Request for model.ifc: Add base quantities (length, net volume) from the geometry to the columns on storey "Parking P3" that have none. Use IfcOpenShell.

First a look at what the model holds.

```python
import ifcopenshell
import ifcopenshell.util.element
import ifcopenshell.util.unit

model = ifcopenshell.open("model.ifc")
print(model.schema)
for unit_type in ("LENGTHUNIT", "AREAUNIT", "VOLUMEUNIT"):
    print(unit_type, ifcopenshell.util.unit.calculate_unit_scale(model, unit_type))
storey = next(s for s in model.by_type("IfcBuildingStorey") if s.Name == "Parking P3")
columns = [e for e in ifcopenshell.util.element.get_decomposition(storey) if e.is_a("IfcColumn")]
for e in sorted(columns, key=lambda e: e.id()):
    print(e.id(), e.is_a(), e.Name, list(ifcopenshell.util.element.get_psets(e, qtos_only=True)), sep=" | ")
```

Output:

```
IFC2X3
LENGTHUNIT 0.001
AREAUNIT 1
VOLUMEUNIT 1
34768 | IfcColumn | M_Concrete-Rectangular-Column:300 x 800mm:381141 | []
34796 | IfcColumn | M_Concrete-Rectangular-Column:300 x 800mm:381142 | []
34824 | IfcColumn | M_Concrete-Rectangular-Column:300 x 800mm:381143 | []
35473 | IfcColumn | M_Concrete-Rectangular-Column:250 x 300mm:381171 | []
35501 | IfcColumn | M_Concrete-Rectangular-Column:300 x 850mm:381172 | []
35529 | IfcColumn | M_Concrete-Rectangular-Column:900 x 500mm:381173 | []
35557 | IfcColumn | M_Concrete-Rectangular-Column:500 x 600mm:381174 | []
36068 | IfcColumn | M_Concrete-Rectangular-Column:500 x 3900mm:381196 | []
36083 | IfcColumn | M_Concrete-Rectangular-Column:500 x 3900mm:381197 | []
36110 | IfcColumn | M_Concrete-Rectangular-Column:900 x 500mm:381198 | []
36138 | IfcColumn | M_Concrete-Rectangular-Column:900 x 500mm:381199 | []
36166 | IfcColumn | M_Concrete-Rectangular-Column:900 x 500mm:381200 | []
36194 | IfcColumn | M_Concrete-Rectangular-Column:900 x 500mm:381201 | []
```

```python
import ifcopenshell
import ifcopenshell.api.pset
import ifcopenshell.geom
import ifcopenshell.util.element
import ifcopenshell.util.shape
import ifcopenshell.util.unit

model = ifcopenshell.open("model.ifc")
unit_scale = ifcopenshell.util.unit.calculate_unit_scale(model)
volume_scale = ifcopenshell.util.unit.calculate_unit_scale(model, "VOLUMEUNIT")
settings = ifcopenshell.geom.settings()

storey = next(s for s in model.by_type("IfcBuildingStorey") if s.Name == "Parking P3")
columns = [e for e in ifcopenshell.util.element.get_decomposition(storey) if e.is_a("IfcColumn")]

for e in sorted(columns, key=lambda e: e.id()):
    if ifcopenshell.util.element.get_psets(e, qtos_only=True, should_inherit=False):
        continue
    # Geometry comes back in metres, in the element's own axes.
    shape = ifcopenshell.geom.create_shape(settings, e)
    values = {
        "Length": ifcopenshell.util.shape.get_z(shape.geometry) / unit_scale,
        "NetVolume": ifcopenshell.util.shape.get_volume(shape.geometry) / volume_scale,
    }
    qto = ifcopenshell.api.pset.add_qto(model, product=e, name="BaseQuantities")
    ifcopenshell.api.pset.edit_qto(model, qto=qto, properties=values)
    print(e.id(), {k: round(v, 3) for k, v in values.items()})

model.write("model_edited.ifc")
```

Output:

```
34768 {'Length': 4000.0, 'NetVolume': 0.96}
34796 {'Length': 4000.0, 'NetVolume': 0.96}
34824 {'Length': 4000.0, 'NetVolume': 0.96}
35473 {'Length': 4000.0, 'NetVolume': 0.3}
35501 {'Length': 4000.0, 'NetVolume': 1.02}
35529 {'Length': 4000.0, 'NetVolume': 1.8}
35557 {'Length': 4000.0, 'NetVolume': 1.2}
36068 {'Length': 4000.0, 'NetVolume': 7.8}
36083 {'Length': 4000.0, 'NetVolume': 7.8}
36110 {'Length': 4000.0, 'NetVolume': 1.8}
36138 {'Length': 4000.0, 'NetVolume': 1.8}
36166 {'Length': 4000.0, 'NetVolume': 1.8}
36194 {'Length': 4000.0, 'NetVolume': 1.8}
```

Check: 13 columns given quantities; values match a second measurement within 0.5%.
